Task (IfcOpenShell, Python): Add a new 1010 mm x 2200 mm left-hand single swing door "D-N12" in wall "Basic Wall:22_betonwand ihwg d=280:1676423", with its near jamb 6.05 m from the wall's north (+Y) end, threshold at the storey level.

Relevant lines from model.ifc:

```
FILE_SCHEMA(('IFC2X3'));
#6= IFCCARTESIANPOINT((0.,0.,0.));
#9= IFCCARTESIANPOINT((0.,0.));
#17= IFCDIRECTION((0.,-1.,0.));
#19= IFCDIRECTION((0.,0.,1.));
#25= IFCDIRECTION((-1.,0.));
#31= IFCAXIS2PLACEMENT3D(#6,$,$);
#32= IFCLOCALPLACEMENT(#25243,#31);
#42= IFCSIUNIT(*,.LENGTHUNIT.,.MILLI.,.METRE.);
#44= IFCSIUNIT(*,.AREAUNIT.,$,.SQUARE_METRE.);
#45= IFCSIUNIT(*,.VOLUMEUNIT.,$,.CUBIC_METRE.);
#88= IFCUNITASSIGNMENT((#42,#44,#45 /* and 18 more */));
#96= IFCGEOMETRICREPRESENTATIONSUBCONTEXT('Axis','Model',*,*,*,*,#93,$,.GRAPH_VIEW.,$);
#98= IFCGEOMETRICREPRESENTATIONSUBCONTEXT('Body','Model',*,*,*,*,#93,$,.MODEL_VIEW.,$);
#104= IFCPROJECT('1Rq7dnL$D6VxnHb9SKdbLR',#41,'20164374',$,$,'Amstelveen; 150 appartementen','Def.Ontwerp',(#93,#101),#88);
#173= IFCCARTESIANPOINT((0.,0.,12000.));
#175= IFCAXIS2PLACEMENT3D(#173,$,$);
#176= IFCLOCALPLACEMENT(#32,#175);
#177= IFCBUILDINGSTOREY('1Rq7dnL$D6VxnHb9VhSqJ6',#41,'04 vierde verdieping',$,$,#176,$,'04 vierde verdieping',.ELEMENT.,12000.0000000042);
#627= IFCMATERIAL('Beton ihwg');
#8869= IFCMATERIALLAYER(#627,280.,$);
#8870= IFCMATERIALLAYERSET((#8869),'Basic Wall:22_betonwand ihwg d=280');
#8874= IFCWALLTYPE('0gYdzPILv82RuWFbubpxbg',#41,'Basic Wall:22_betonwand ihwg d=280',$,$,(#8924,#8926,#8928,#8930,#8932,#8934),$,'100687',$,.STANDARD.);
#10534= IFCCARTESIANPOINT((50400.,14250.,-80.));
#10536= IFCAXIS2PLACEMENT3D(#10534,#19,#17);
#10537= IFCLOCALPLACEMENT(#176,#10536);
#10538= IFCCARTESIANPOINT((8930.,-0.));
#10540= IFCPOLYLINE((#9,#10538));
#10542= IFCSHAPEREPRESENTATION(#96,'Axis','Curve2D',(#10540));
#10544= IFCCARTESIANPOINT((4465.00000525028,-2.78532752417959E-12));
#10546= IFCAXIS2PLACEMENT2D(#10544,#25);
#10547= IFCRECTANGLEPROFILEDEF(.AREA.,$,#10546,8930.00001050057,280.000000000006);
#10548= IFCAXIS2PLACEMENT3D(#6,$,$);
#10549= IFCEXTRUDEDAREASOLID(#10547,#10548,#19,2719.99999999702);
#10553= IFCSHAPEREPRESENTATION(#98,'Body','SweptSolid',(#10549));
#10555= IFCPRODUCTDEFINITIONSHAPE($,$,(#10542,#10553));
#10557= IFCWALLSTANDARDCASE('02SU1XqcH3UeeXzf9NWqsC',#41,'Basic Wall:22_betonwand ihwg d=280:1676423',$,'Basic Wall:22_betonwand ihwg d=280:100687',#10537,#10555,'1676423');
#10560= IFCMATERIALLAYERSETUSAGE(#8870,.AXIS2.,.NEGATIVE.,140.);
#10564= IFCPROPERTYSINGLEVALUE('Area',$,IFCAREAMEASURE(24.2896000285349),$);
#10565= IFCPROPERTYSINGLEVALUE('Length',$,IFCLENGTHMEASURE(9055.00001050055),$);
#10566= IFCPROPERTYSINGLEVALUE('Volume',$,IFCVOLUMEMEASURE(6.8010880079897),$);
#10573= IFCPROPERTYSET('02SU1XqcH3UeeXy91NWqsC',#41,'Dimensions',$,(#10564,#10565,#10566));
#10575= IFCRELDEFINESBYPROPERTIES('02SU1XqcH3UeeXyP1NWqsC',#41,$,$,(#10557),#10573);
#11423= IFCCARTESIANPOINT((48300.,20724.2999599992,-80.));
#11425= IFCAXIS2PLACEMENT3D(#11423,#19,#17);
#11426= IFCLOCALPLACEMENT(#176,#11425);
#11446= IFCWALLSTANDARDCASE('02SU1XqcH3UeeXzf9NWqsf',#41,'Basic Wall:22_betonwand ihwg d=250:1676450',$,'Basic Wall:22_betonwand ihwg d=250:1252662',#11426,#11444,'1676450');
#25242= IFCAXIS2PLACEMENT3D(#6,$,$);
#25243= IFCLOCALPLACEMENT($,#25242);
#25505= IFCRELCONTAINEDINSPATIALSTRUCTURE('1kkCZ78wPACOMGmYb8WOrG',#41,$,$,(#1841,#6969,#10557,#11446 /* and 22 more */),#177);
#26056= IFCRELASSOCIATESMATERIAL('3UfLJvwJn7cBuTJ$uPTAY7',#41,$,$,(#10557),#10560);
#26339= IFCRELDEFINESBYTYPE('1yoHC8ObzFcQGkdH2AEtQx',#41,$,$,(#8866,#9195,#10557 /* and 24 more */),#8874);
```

```python
import numpy as np
import ifcopenshell
import ifcopenshell.api.feature
import ifcopenshell.api.geometry
import ifcopenshell.api.pset
import ifcopenshell.api.root
import ifcopenshell.api.spatial
import ifcopenshell.api.type
import ifcopenshell.geom
import ifcopenshell.util.element
import ifcopenshell.util.placement
import ifcopenshell.util.representation
import ifcopenshell.util.shape
import ifcopenshell.util.unit

model = ifcopenshell.open("model.ifc")
unit_scale = ifcopenshell.util.unit.calculate_unit_scale(model)
area_scale = ifcopenshell.util.unit.calculate_unit_scale(model, "AREAUNIT")
volume_scale = ifcopenshell.util.unit.calculate_unit_scale(model, "VOLUMEUNIT")
settings = ifcopenshell.geom.settings()


def volume(element):
    """Net volume in cubic metres, openings subtracted."""
    shape = ifcopenshell.geom.create_shape(settings, element)
    return ifcopenshell.util.shape.get_volume(shape.geometry)


wall = model.by_id(10557)
storey = ifcopenshell.util.element.get_container(wall, ifc_class="IfcBuildingStorey")
context = ifcopenshell.util.representation.get_context(model, "Model", "Body", "MODEL_VIEW")
before = volume(wall)

width, height, from_end, sill = 1.01, 2.2, 6.05, 0.0  # metres

# The wall runs along its own X axis, and the end named is its -X end.
wall_shape = ifcopenshell.geom.create_shape(settings, wall)
x, y, z = ifcopenshell.util.shape.get_vertices(wall_shape.geometry).T
start = x.min() + from_end
face, thickness = float(y.min()), float(y.max() - y.min())
wall_matrix = ifcopenshell.util.placement.get_local_placement(wall.ObjectPlacement)
level = ifcopenshell.util.placement.get_local_placement(storey.ObjectPlacement)[2, 3]


def in_wall(x, y):
    """Placement at x, y metres in the wall's axes, at sill height."""
    matrix = wall_matrix.copy()
    matrix[:, 3] = wall_matrix @ np.array([x / unit_scale, y / unit_scale, 0.0, 1.0])
    matrix[2, 3] = level + sill / unit_scale
    return matrix


# Opening: a box that overshoots both wall faces by 50 mm.
opening = ifcopenshell.api.root.create_entity(model, ifc_class="IfcOpeningElement")
box = ifcopenshell.api.geometry.add_wall_representation(
    model, context=context, length=width, height=height, thickness=thickness + 0.1
)
ifcopenshell.api.geometry.assign_representation(model, product=opening, representation=box)
ifcopenshell.api.geometry.edit_object_placement(model, product=opening, matrix=in_wall(start, face - 0.05), is_si=False)
ifcopenshell.api.feature.add_feature(model, feature=opening, element=wall)

door = ifcopenshell.api.root.create_entity(model, ifc_class="IfcDoor", name="D-N12")
door.OverallWidth, door.OverallHeight = width / unit_scale, height / unit_scale
body = ifcopenshell.api.geometry.add_door_representation(
    model,
    context=context,
    overall_width=door.OverallWidth,
    overall_height=door.OverallHeight,
    operation_type="SINGLE_SWING_LEFT",
    lining_properties={"LiningDepth": thickness / unit_scale, "ThresholdDepth": thickness / unit_scale},
)
ifcopenshell.api.geometry.assign_representation(model, product=door, representation=body)
ifcopenshell.api.spatial.assign_container(model, products=[door], relating_structure=storey)
fills = ifcopenshell.api.feature.add_filling(model, opening=opening, element=door)
fills.OwnerHistory = door.OwnerHistory  # required in IFC2X3

# IFC2X3 keeps the operation on the door style.
style = ifcopenshell.api.root.create_entity(model, ifc_class="IfcDoorStyle", name="D-N12")
style.OperationType, style.ConstructionType = "SINGLE_SWING_LEFT", "NOTDEFINED"
style.ParameterTakesPrecedence = style.Sizeable = False
ifcopenshell.api.type.assign_type(model, related_objects=[door], relating_type=style)

# The lining spans the wall, so the door starts at the wall face.
ifcopenshell.api.geometry.edit_object_placement(model, product=door, matrix=in_wall(start, face), is_si=False)

after = volume(wall)

# Update the wall's stored quantities.
pset = model.by_id(ifcopenshell.util.element.get_pset(wall, "Dimensions", should_inherit=False)["id"])
ifcopenshell.api.pset.edit_pset(model, pset=pset, properties={
    "Area": model.create_entity("IfcAreaMeasure", after / thickness / area_scale),
    "Volume": model.create_entity("IfcVolumeMeasure", after / volume_scale),
})

print(f"wall volume {before:.3f} -> {after:.3f} m3")

model.write("model_edited.ifc")
```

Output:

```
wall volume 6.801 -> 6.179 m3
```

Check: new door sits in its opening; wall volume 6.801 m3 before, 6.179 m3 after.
